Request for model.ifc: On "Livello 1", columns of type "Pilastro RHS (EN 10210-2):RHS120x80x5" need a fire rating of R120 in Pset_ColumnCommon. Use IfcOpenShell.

First a look at what the model holds.

```python
import ifcopenshell
import ifcopenshell.util.element

model = ifcopenshell.open("model.ifc")
print(model.schema)
storey = next(s for s in model.by_type("IfcBuildingStorey") if s.Name == "Livello 1")
columns = [e for e in ifcopenshell.util.element.get_decomposition(storey) if e.is_a("IfcColumn")]
seen = {}
for e in columns:
    element_type = ifcopenshell.util.element.get_type(e)
    key = (element_type.Name if element_type != e and element_type else None, ifcopenshell.util.element.get_pset(e, "Pset_ColumnCommon", "FireRating"))
    seen[key] = seen.get(key, 0) + 1
for (name, value), count in sorted(seen.items(), key=str):
    print(count, "x", name, "|", value)
```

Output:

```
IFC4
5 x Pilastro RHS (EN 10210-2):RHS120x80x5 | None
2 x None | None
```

```python
import ifcopenshell
import ifcopenshell.api.pset
import ifcopenshell.util.element

model = ifcopenshell.open("model.ifc")

storey = next(s for s in model.by_type("IfcBuildingStorey") if s.Name == "Livello 1")
columns = [e for e in ifcopenshell.util.element.get_decomposition(storey) if e.is_a("IfcColumn")]

count = 0
for e in columns:
    element_type = ifcopenshell.util.element.get_type(e)
    if element_type in (None, e) or element_type.Name != "Pilastro RHS (EN 10210-2):RHS120x80x5":
        continue
    # add_pset returns the element's existing set when there is one.
    pset = ifcopenshell.api.pset.add_pset(model, product=e, name="Pset_ColumnCommon")
    ifcopenshell.api.pset.edit_pset(model, pset=pset, properties={"FireRating": "R120"})
    count += 1

print(count, "columns updated")

model.write("model_updated.ifc")
```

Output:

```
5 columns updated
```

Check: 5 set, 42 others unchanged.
